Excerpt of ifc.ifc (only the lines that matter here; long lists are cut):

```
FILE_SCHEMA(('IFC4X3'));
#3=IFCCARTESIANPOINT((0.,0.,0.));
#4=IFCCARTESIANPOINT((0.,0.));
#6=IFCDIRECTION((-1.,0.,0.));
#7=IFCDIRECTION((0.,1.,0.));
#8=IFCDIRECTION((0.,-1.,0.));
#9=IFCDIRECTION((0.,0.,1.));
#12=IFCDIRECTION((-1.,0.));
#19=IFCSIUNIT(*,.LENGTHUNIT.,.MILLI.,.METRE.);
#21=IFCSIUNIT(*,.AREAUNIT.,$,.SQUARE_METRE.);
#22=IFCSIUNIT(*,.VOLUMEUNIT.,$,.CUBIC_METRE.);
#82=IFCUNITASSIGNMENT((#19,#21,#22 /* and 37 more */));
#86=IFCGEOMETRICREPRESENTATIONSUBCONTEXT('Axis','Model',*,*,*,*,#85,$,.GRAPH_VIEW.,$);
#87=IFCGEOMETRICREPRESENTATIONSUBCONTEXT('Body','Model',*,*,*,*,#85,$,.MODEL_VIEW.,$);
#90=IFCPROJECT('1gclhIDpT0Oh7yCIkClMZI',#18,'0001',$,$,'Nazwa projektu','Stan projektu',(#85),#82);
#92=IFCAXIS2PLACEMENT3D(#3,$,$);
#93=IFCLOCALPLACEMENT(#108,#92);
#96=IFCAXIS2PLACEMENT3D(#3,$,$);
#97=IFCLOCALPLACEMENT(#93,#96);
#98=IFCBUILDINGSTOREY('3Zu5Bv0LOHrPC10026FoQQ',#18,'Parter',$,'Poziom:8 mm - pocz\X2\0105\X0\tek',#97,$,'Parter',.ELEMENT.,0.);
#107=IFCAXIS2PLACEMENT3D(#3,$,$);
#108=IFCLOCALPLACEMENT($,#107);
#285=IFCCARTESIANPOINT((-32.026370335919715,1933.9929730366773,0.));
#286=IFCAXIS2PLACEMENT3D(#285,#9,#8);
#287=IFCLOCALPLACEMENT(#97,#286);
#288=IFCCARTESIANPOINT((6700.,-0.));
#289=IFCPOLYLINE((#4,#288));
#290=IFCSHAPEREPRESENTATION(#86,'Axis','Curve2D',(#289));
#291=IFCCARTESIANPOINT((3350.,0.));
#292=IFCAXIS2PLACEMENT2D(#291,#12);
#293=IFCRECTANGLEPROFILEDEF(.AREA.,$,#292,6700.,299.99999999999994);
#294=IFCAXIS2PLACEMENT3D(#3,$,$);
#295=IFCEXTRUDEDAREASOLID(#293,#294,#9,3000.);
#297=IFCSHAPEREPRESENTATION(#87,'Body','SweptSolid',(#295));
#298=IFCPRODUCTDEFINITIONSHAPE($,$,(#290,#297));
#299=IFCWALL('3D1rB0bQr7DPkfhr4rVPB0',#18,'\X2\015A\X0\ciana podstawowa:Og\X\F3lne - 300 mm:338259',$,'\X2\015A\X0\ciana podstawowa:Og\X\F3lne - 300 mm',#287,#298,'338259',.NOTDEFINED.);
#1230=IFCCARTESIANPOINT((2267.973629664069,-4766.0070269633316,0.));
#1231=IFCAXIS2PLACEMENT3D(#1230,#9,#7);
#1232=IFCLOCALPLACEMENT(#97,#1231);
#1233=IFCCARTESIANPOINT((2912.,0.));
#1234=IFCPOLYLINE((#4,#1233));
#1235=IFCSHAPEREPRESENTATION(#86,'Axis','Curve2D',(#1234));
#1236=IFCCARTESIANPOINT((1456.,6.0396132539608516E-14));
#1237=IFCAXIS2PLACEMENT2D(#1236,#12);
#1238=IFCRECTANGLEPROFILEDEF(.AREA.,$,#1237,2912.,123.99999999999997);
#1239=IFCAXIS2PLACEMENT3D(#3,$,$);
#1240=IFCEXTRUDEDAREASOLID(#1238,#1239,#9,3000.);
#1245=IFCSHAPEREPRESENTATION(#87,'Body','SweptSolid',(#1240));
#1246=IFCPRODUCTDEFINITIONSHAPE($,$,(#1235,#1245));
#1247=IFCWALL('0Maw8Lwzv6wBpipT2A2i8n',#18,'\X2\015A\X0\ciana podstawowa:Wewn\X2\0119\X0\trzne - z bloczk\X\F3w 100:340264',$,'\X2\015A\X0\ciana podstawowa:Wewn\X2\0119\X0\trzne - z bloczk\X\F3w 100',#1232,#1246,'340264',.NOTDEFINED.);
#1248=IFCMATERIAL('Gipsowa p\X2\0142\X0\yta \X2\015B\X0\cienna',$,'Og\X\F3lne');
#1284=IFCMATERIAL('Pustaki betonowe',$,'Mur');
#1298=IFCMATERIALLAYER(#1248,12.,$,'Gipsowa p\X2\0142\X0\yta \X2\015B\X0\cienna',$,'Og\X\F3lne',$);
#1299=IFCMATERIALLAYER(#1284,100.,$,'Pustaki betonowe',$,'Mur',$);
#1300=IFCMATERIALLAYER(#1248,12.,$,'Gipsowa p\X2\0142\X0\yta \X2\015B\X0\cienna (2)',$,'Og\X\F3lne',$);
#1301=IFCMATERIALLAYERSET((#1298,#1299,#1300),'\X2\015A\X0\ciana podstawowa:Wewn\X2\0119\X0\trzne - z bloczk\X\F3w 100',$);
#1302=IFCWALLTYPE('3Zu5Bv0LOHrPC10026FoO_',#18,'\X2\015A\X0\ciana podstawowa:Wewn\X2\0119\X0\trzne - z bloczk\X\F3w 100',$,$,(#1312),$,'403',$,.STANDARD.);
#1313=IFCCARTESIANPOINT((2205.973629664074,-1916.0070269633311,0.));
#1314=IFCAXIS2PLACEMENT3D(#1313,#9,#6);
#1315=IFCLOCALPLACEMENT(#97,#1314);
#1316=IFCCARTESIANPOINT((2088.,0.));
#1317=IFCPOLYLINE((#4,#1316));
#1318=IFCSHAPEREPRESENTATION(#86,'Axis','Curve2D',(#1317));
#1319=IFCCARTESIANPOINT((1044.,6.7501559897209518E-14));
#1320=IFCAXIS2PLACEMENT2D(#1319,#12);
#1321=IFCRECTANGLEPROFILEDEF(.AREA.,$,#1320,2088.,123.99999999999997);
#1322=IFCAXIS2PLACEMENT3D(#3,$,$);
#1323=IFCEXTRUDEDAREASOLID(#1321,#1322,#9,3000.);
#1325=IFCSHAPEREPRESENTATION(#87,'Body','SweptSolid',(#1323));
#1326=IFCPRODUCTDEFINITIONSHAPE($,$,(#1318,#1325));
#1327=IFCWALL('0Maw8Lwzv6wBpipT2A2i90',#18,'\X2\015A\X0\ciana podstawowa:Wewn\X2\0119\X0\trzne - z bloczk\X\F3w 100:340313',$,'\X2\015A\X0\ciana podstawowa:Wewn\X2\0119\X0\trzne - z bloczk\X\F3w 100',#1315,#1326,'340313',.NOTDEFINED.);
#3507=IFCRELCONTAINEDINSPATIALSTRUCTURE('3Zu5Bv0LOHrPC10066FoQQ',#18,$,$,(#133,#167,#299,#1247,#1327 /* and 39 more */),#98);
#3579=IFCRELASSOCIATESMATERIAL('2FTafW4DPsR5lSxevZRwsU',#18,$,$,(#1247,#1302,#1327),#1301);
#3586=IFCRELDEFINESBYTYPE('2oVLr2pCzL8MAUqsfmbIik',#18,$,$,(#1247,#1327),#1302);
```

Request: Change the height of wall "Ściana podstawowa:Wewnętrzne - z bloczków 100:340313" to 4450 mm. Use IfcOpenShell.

```python
import ifcopenshell
import ifcopenshell.geom
import ifcopenshell.util.representation
import ifcopenshell.util.shape

model = ifcopenshell.open("ifc.ifc")
settings = ifcopenshell.geom.settings()


def volume(element):
    """Net volume in cubic metres, openings subtracted."""
    shape = ifcopenshell.geom.create_shape(settings, element)
    return ifcopenshell.util.shape.get_volume(shape.geometry)


wall = model.by_id(1327)
before = volume(wall)

body = ifcopenshell.util.representation.get_representation(wall, "Model", "Body")
solid = body.Items[0]
old_height = solid.Depth
solid.Depth = 4450.0
after = volume(wall)

print(f"height {old_height:g} -> {solid.Depth:g}, volume {before:.3f} -> {after:.3f} m3")

model.write("ifc_updated.ifc")
```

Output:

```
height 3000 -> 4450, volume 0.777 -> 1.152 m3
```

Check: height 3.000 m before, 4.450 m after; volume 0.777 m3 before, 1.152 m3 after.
